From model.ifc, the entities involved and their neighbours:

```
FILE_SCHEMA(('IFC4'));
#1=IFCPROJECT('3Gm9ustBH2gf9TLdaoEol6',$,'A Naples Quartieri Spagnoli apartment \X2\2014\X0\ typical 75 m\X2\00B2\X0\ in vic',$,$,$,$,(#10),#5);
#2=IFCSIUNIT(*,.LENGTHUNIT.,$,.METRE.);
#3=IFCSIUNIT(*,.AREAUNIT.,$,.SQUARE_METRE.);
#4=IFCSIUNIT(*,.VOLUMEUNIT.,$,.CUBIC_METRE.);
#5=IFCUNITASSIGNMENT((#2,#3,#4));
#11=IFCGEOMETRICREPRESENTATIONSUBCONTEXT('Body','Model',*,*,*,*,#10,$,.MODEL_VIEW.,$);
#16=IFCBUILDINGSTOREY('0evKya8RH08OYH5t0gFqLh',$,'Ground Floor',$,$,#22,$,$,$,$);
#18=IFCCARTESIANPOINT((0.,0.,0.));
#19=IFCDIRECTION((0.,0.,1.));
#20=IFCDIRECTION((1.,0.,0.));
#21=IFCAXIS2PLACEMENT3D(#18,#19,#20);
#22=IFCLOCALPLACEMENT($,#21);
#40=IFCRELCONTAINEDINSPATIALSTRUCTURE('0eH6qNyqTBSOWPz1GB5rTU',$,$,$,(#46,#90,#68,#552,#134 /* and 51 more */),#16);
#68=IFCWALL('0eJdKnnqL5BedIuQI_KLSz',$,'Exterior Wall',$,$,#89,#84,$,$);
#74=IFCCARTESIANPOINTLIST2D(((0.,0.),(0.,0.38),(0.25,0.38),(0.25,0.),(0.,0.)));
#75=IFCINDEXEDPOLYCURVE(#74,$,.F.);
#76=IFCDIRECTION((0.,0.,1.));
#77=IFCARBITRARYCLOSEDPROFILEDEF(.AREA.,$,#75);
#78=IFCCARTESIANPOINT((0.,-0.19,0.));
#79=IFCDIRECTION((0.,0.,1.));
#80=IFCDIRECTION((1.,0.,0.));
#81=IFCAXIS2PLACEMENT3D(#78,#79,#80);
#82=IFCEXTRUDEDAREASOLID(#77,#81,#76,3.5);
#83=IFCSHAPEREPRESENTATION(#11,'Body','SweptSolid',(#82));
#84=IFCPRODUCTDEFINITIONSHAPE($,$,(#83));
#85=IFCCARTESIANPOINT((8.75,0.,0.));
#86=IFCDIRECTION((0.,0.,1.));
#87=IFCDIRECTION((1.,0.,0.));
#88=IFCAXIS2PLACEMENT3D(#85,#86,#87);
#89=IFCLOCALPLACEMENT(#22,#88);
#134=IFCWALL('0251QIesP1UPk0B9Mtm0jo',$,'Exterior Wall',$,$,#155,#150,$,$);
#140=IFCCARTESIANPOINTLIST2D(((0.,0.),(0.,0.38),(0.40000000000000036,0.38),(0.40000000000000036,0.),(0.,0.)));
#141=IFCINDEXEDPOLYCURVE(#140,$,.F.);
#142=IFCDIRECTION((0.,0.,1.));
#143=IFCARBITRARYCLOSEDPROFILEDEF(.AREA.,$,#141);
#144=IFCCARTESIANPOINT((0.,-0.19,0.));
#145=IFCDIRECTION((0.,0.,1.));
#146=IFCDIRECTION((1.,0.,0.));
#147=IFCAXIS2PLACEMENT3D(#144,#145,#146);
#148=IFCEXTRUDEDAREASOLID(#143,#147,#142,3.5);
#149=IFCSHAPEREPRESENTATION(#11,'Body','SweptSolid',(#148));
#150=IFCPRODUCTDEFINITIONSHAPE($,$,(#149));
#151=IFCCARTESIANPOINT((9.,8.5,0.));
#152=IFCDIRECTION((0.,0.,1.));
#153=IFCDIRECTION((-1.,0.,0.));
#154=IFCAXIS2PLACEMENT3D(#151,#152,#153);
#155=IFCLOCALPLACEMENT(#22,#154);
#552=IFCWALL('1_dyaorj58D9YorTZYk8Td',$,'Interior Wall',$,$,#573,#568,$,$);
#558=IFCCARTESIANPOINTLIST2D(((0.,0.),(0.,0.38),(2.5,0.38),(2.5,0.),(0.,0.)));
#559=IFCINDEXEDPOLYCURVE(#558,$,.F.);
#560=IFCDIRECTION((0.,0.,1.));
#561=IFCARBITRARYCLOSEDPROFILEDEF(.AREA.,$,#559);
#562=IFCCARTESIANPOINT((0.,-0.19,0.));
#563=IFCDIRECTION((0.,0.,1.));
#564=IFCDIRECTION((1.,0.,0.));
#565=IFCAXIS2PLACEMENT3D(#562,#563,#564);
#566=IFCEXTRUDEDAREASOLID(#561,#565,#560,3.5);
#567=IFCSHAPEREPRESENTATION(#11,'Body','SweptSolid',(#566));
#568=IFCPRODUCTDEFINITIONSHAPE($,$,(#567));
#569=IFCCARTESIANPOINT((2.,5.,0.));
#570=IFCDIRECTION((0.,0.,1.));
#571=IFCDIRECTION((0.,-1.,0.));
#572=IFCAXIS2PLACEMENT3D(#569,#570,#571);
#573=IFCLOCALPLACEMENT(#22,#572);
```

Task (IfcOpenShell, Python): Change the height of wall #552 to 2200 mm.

```python
import ifcopenshell
import ifcopenshell.geom
import ifcopenshell.util.representation
import ifcopenshell.util.shape
import ifcopenshell.util.unit

model = ifcopenshell.open("model.ifc")
unit_scale = ifcopenshell.util.unit.calculate_unit_scale(model)
settings = ifcopenshell.geom.settings()


def volume(element):
    """Net volume in cubic metres, openings subtracted."""
    shape = ifcopenshell.geom.create_shape(settings, element)
    return ifcopenshell.util.shape.get_volume(shape.geometry)


wall = model.by_guid("1_dyaorj58D9YorTZYk8Td")
before = volume(wall)

body = ifcopenshell.util.representation.get_representation(wall, "Model", "Body")
solid = body.Items[0]
old_height = solid.Depth
solid.Depth = 2.2 / unit_scale
after = volume(wall)

print(f"height {old_height:g} -> {solid.Depth:g}, volume {before:.3f} -> {after:.3f} m3")

model.write("model_updated.ifc")
```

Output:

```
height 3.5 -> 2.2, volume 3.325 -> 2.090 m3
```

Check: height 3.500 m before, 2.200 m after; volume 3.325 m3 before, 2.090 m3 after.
